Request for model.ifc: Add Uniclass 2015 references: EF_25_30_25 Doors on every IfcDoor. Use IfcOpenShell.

First a look at what the model holds.

```python
import ifcopenshell

model = ifcopenshell.open("model.ifc")
print(model.schema)
print("classifications:", [c.Name for c in model.by_type("IfcClassification")])
for ifc_class in ("IfcDoor", "IfcRoof", "IfcStair", "IfcWall", "IfcWindow"):
    print(ifc_class, len(model.by_type(ifc_class)))
```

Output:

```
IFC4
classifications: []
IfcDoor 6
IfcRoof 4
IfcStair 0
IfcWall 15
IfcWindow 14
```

```python
import ifcopenshell
import ifcopenshell.api.classification

model = ifcopenshell.open("model.ifc")

system = ifcopenshell.api.classification.add_classification(model, classification="Uniclass 2015")

codes = {
    "IfcDoor": ("EF_25_30_25", "Doors"),
}
for ifc_class, (code, name) in codes.items():
    products = model.by_type(ifc_class)
    ifcopenshell.api.classification.add_reference(
        model, products=products, classification=system, identification=code, name=name
    )
    print(code, len(products))

model.write("model_edited.ifc")
```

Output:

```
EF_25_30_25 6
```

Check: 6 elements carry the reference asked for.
